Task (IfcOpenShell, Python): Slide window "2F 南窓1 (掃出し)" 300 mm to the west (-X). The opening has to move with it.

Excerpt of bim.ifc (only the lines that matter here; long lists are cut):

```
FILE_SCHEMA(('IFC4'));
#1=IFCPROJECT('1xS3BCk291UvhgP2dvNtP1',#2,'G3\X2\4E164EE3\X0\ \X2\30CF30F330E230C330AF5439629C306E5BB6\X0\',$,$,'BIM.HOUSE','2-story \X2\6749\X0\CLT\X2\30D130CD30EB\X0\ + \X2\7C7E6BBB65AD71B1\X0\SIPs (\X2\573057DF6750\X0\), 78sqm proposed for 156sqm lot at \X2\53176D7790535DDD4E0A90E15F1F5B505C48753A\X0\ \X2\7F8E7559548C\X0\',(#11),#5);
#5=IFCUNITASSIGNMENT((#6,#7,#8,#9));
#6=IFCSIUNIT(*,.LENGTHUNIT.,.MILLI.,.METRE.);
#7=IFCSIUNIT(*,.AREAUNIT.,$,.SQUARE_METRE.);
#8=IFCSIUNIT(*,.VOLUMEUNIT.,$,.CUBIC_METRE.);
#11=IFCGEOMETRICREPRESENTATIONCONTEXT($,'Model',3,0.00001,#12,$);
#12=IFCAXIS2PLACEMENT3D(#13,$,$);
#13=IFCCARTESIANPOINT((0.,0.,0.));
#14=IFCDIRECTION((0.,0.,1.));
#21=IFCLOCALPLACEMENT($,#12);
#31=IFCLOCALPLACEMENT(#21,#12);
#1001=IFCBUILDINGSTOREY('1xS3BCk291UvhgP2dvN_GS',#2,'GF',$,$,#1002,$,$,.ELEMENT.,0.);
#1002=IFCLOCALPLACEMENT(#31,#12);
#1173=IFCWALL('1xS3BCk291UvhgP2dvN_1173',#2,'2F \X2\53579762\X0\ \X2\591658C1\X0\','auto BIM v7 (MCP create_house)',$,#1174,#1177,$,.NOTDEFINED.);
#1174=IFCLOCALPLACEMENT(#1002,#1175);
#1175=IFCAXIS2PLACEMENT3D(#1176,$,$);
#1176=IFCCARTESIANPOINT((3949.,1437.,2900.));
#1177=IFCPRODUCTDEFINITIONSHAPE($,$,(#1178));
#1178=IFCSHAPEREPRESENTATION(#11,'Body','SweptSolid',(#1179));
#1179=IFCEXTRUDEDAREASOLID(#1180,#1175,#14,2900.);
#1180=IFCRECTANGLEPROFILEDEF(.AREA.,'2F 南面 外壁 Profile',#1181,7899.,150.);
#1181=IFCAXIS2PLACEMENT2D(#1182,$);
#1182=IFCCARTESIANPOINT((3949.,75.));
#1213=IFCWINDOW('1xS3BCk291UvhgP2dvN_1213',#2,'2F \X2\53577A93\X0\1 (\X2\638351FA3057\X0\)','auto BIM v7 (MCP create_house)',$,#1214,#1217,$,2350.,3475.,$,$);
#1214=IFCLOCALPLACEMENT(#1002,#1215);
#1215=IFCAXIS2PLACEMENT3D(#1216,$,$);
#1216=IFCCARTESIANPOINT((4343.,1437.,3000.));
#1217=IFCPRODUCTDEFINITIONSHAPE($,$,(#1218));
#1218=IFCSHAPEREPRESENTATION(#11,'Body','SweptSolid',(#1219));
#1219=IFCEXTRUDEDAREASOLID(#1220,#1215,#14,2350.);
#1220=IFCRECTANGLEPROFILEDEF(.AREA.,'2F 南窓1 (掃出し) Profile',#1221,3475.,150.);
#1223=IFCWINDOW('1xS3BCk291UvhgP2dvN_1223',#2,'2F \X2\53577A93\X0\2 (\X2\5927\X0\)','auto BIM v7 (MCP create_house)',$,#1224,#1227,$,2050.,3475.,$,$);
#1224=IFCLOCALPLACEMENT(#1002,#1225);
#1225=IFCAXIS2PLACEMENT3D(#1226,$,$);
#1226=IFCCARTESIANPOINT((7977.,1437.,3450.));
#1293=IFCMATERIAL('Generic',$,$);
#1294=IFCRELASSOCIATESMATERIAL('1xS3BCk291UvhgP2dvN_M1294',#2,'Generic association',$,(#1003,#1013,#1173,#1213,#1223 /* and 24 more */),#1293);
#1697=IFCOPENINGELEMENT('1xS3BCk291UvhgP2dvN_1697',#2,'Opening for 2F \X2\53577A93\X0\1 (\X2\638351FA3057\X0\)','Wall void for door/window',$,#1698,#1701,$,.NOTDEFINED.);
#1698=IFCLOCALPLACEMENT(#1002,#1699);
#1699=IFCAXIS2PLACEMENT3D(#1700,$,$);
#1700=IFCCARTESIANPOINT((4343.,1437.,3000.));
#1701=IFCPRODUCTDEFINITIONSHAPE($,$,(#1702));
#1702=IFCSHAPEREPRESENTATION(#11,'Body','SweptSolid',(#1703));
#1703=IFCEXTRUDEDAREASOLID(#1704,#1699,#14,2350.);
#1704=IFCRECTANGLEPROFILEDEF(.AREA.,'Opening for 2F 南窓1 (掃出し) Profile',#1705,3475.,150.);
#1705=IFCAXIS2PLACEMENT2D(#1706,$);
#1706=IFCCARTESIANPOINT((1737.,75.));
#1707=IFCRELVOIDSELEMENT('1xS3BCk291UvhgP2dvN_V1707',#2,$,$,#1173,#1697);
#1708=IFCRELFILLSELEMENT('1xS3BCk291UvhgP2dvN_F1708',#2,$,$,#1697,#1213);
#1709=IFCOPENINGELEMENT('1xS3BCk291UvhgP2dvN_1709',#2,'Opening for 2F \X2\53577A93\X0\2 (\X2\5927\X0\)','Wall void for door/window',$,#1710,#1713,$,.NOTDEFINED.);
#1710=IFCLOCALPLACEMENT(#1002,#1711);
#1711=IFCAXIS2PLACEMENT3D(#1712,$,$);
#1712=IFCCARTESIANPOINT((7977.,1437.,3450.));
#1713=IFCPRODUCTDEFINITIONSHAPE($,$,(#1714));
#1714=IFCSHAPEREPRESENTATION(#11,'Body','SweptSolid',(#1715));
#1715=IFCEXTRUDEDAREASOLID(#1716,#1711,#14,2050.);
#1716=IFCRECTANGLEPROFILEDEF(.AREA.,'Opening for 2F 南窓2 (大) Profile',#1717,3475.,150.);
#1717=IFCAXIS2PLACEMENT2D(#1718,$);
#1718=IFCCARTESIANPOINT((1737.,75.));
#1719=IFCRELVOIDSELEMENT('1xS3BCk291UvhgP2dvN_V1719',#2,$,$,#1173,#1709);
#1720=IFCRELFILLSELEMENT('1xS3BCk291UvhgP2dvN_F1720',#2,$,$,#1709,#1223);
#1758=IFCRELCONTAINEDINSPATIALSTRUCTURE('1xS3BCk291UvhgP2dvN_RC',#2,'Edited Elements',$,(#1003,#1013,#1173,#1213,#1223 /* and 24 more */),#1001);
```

```python
import ifcopenshell
import ifcopenshell.api.geometry
import ifcopenshell.util.placement

model = ifcopenshell.open("bim.ifc")

window = model.by_guid("1xS3BCk291UvhgP2dvN_1213")
opening = window.FillsVoids[0].RelatingOpeningElement
wall = opening.VoidsElements[0].RelatingBuildingElement

wall_matrix = ifcopenshell.util.placement.get_local_placement(wall.ObjectPlacement)
shift = wall_matrix[:3, 0] * -300.0
before = ifcopenshell.util.placement.get_local_placement(window.ObjectPlacement)[:3, 3].copy()

# The window is not placed relative to its opening, so move both.
for product in (opening, window):
    matrix = ifcopenshell.util.placement.get_local_placement(product.ObjectPlacement)
    matrix[:3, 3] += shift
    ifcopenshell.api.geometry.edit_object_placement(model, product=product, matrix=matrix, is_si=False)

after = ifcopenshell.util.placement.get_local_placement(window.ObjectPlacement)[:3, 3]
print("window moved by", (after - before).round(3) + 0.0)

model.write("bim-out.ifc")
```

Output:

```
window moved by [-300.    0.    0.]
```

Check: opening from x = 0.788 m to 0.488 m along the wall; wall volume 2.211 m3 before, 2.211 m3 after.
